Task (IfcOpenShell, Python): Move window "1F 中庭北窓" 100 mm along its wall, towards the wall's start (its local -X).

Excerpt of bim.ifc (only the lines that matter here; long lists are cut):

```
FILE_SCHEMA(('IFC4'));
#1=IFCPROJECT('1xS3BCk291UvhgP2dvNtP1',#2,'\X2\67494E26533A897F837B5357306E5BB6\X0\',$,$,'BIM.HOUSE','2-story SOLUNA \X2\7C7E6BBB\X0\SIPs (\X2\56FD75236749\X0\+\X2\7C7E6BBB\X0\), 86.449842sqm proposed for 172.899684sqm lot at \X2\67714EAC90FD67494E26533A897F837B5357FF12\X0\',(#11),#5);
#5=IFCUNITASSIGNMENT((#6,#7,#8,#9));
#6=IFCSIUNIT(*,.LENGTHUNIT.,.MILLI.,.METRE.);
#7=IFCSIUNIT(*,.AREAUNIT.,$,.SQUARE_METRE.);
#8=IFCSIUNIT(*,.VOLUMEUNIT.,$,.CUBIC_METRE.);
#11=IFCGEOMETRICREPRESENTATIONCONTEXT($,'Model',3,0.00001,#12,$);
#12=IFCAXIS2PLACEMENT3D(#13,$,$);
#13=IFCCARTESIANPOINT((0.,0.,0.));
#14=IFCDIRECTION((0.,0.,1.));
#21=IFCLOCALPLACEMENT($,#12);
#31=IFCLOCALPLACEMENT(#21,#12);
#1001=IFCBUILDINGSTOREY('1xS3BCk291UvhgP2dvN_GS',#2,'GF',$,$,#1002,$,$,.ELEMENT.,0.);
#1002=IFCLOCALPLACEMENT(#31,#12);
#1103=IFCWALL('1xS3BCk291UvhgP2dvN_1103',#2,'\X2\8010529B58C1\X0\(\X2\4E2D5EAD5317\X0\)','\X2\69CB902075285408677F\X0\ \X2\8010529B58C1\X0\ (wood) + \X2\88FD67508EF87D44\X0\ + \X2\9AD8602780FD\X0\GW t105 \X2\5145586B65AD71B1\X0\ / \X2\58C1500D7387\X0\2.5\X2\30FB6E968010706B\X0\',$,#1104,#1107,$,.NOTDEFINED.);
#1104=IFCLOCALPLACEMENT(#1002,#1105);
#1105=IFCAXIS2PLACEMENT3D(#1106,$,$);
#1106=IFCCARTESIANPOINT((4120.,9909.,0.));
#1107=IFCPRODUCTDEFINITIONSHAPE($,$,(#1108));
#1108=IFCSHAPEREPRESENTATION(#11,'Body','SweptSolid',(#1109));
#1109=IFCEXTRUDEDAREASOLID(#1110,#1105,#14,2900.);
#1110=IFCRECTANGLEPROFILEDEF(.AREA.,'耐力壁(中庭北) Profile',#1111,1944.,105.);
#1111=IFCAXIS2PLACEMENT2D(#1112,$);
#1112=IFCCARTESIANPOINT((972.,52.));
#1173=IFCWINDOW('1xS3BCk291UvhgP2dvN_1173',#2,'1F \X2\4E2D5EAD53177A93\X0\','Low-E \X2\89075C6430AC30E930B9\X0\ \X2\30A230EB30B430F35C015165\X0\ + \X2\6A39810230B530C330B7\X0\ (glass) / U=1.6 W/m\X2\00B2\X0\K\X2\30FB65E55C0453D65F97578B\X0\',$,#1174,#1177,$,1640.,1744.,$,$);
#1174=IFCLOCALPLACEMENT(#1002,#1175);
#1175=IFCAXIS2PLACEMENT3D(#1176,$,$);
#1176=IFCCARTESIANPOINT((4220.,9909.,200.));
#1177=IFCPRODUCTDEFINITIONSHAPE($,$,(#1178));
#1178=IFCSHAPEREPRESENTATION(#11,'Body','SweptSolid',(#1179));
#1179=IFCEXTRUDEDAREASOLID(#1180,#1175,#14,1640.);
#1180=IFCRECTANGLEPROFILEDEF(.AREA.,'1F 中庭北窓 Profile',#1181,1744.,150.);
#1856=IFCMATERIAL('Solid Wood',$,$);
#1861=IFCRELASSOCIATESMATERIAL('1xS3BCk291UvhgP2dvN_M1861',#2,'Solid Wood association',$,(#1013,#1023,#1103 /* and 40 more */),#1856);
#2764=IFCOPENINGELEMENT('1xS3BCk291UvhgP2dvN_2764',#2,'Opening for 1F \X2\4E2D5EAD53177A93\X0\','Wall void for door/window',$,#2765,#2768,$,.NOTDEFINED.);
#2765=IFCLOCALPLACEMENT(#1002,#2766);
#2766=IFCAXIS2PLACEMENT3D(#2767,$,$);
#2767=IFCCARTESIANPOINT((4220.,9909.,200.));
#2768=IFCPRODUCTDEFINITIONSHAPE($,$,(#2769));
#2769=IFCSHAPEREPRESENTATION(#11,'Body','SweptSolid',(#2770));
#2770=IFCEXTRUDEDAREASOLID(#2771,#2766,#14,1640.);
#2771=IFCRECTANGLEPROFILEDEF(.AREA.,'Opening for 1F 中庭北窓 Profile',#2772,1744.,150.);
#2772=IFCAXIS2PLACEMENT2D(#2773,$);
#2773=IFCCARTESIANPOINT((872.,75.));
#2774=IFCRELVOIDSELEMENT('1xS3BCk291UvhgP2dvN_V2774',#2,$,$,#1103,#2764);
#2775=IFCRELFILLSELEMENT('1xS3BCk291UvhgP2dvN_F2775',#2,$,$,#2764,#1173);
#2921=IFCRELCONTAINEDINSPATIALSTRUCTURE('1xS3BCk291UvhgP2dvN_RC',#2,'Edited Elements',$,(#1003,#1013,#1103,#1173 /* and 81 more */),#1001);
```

```python
import ifcopenshell
import ifcopenshell.api.geometry
import ifcopenshell.util.placement
import ifcopenshell.util.unit

model = ifcopenshell.open("bim.ifc")
unit_scale = ifcopenshell.util.unit.calculate_unit_scale(model)

window = model.by_guid("1xS3BCk291UvhgP2dvN_1173")
opening = window.FillsVoids[0].RelatingOpeningElement
wall = opening.VoidsElements[0].RelatingBuildingElement

wall_matrix = ifcopenshell.util.placement.get_local_placement(wall.ObjectPlacement)
shift = wall_matrix[:3, 0] * -0.1 / unit_scale
before = ifcopenshell.util.placement.get_local_placement(window.ObjectPlacement)[:3, 3].copy()

# The window is not placed relative to its opening, so move both.
for product in (opening, window):
    matrix = ifcopenshell.util.placement.get_local_placement(product.ObjectPlacement)
    matrix[:3, 3] += shift
    ifcopenshell.api.geometry.edit_object_placement(model, product=product, matrix=matrix, is_si=False)

after = ifcopenshell.util.placement.get_local_placement(window.ObjectPlacement)[:3, 3]
print("window moved by", (after - before).round(3) + 0.0)

model.write("bim_edited.ifc")
```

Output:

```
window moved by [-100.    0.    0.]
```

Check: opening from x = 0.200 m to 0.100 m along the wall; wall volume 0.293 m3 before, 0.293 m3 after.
